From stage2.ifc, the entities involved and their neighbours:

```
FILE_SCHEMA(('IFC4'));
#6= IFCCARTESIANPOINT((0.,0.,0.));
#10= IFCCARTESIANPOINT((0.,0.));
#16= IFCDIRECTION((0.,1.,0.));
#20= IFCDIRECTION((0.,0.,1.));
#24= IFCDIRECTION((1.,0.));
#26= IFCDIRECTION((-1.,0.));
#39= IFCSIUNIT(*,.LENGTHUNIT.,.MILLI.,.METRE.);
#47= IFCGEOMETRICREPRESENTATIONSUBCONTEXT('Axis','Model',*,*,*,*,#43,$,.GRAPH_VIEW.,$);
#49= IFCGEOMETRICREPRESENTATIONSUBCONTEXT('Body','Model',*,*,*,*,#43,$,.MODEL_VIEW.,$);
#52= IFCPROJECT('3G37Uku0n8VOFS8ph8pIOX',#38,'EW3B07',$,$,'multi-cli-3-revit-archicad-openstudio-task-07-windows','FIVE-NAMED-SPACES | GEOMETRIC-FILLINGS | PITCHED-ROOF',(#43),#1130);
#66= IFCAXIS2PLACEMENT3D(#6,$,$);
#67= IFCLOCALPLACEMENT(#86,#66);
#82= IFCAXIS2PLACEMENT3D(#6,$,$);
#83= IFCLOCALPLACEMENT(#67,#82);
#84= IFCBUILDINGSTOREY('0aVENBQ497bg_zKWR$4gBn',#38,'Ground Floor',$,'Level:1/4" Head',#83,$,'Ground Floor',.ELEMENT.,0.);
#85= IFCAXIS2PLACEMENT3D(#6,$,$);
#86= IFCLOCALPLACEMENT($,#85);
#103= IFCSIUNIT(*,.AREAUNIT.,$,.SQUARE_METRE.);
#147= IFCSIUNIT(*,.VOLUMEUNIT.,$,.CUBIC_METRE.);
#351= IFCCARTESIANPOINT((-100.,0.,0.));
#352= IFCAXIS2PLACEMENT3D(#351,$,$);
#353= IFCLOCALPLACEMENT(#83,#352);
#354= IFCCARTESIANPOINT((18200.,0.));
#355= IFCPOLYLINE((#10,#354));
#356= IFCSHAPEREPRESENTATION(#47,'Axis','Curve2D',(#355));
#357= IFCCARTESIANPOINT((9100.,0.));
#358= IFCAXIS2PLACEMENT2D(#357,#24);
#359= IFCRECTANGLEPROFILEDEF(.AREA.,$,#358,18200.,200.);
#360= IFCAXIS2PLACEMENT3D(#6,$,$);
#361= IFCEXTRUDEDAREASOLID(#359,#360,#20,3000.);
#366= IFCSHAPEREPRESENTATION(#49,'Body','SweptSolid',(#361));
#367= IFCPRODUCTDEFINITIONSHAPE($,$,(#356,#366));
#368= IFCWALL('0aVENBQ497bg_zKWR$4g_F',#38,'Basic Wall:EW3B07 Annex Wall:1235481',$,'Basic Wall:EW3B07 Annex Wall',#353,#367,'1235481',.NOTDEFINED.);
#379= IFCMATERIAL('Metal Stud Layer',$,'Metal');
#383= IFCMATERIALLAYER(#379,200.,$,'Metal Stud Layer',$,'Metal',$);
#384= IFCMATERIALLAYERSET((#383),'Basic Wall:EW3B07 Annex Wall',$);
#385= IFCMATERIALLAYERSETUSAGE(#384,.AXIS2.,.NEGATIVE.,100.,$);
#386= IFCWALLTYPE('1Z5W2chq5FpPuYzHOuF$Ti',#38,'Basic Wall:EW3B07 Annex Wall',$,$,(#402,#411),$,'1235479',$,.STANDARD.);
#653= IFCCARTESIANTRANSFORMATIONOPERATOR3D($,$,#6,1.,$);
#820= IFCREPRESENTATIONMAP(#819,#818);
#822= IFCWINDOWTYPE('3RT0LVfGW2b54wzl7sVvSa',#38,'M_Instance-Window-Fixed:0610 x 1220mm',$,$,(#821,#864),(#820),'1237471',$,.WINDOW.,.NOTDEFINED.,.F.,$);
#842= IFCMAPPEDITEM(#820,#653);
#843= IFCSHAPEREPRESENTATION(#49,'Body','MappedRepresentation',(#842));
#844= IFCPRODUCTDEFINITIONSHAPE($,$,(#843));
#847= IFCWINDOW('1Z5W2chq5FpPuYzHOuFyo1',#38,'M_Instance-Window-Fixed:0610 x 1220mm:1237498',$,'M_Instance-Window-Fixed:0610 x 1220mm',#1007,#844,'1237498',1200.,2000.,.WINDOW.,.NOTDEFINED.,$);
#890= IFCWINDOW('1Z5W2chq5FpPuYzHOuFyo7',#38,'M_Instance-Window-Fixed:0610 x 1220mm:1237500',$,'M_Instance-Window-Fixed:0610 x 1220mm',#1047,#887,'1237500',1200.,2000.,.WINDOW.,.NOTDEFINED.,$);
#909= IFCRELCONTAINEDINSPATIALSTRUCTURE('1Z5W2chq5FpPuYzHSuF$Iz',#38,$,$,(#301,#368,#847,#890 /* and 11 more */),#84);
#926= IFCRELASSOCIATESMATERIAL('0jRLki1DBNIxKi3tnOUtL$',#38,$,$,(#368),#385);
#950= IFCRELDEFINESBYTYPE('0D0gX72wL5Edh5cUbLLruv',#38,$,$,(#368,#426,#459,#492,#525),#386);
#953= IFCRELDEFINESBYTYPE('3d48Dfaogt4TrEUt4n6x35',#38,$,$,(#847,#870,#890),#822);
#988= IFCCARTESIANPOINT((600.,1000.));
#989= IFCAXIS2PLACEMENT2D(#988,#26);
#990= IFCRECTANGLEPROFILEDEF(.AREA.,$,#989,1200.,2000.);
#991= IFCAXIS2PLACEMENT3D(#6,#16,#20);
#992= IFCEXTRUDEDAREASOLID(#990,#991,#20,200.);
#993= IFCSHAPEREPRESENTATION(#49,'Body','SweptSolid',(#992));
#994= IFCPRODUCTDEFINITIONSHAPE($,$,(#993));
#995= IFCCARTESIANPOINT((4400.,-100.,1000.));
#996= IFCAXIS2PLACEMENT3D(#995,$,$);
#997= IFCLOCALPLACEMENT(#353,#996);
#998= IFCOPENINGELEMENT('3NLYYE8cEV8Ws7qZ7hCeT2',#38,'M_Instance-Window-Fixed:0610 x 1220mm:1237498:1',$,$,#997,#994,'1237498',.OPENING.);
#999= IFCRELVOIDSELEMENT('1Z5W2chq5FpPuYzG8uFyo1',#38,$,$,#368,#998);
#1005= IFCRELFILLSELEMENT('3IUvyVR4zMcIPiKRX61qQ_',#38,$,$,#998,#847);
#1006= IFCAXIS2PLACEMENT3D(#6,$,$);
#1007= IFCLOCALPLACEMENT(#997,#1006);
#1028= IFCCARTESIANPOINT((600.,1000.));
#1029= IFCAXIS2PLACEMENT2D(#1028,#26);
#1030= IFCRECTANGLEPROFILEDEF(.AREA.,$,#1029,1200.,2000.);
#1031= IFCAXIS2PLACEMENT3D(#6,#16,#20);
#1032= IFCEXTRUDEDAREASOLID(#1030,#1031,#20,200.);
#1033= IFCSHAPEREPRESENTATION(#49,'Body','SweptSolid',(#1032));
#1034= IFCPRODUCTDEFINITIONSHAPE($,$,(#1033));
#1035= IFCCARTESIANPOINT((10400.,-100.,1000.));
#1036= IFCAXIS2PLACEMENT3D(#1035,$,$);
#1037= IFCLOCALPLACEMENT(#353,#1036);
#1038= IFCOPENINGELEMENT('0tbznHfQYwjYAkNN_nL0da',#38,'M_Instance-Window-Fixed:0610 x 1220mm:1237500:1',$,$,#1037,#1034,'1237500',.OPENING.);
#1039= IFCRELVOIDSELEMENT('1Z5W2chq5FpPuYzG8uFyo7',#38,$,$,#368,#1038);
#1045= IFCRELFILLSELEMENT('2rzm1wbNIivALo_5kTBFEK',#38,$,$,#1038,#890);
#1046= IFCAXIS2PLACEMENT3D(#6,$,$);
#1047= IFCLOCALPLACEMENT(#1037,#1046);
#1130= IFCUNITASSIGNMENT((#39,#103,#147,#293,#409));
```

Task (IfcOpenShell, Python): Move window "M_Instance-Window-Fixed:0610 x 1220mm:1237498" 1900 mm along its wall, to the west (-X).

```python
import ifcopenshell
import ifcopenshell.api.geometry
import ifcopenshell.util.placement
import ifcopenshell.util.unit

model = ifcopenshell.open("stage2.ifc")
unit_scale = ifcopenshell.util.unit.calculate_unit_scale(model)

window = model.by_guid("1Z5W2chq5FpPuYzHOuFyo1")
opening = window.FillsVoids[0].RelatingOpeningElement
wall = opening.VoidsElements[0].RelatingBuildingElement

wall_matrix = ifcopenshell.util.placement.get_local_placement(wall.ObjectPlacement)
shift = wall_matrix[:3, 0] * -1.9 / unit_scale
before = ifcopenshell.util.placement.get_local_placement(window.ObjectPlacement)[:3, 3].copy()

# The window is placed relative to its opening, so it follows when the opening moves.
matrix = ifcopenshell.util.placement.get_local_placement(opening.ObjectPlacement)
matrix[:3, 3] += shift
ifcopenshell.api.geometry.edit_object_placement(
    model, product=opening, matrix=matrix, is_si=False, should_transform_children=True
)

after = ifcopenshell.util.placement.get_local_placement(window.ObjectPlacement)[:3, 3]
print("window moved by", (after - before).round(3) + 0.0)

model.write("stage2_rev.ifc")
```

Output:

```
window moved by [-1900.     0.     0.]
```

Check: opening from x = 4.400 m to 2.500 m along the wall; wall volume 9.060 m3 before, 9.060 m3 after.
